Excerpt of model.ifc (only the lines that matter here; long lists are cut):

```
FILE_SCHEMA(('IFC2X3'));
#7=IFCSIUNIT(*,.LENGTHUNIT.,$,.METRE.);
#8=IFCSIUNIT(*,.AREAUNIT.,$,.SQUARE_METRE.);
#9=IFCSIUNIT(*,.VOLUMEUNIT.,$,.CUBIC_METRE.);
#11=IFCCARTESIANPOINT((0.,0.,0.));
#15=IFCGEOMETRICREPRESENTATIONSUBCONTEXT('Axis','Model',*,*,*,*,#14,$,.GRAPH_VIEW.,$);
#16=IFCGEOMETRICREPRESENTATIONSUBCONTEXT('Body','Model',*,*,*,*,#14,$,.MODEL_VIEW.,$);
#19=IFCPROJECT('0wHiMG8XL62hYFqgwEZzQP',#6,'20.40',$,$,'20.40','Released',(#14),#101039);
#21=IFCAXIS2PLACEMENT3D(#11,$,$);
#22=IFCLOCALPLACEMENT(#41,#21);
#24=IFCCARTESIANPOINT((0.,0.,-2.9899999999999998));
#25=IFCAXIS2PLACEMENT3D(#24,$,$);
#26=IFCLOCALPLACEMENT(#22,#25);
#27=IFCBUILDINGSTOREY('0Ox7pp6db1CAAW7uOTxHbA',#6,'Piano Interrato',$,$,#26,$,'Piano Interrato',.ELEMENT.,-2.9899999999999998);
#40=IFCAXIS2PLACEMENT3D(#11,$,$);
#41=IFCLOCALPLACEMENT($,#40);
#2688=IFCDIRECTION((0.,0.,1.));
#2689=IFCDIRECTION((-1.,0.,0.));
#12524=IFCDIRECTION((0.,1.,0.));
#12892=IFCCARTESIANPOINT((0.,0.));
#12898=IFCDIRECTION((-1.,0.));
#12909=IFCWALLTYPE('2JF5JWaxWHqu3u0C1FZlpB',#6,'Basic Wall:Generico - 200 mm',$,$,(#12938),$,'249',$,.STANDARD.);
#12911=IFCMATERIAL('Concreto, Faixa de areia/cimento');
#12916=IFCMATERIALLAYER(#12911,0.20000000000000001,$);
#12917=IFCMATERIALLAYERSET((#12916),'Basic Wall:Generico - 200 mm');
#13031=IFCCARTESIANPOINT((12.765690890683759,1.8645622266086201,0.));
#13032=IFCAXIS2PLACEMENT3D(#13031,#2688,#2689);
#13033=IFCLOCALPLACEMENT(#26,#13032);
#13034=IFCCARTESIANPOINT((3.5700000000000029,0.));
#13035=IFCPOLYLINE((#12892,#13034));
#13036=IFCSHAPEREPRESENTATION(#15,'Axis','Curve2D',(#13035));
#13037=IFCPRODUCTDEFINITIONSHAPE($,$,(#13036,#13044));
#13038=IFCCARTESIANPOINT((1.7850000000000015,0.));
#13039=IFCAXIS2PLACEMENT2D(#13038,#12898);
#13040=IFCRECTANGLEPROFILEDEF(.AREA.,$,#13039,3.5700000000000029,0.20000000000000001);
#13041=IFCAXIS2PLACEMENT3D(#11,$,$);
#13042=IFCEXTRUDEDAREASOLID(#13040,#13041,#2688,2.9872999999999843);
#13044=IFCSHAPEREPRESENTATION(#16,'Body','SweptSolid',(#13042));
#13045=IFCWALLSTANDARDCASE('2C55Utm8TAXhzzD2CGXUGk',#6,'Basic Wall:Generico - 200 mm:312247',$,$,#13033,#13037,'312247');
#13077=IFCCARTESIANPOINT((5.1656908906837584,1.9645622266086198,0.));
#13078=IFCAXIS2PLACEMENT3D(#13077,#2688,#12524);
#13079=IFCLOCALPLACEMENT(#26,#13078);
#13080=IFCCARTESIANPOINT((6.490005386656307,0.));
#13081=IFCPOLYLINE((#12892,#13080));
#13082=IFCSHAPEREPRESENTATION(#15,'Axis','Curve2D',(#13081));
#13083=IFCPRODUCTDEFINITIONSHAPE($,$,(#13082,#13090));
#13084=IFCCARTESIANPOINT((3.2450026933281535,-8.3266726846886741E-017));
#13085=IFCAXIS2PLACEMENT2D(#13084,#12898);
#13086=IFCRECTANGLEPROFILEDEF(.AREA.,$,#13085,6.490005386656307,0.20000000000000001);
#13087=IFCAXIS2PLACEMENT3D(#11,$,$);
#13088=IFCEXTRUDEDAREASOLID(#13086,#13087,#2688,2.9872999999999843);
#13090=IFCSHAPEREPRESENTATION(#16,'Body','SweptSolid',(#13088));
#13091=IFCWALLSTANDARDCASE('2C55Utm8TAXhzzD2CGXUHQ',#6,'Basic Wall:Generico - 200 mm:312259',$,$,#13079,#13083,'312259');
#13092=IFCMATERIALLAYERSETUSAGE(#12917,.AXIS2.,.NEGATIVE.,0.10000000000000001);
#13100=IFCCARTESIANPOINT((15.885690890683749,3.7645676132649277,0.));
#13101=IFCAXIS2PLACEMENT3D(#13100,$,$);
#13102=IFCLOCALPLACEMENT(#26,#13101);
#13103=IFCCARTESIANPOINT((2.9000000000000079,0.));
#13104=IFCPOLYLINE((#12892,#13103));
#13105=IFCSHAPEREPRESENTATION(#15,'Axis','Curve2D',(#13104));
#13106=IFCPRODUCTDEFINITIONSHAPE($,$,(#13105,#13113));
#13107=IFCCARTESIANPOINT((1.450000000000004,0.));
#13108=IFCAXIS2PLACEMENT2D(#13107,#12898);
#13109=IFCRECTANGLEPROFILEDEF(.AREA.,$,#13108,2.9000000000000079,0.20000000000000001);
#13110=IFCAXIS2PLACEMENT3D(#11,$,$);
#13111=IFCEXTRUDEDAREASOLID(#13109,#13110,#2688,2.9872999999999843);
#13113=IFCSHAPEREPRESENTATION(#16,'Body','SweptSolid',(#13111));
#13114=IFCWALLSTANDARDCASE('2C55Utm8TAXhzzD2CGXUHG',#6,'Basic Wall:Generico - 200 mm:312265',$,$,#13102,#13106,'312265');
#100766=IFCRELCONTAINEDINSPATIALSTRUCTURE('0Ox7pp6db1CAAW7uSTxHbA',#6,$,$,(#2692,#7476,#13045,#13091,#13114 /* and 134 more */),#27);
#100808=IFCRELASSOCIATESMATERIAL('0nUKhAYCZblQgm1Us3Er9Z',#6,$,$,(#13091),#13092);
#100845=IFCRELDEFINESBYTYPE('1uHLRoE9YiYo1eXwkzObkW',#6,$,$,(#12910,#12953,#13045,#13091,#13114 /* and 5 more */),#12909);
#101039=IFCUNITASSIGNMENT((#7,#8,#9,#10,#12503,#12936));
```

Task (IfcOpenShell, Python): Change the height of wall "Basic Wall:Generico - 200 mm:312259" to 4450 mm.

```python
import ifcopenshell
import ifcopenshell.geom
import ifcopenshell.util.representation
import ifcopenshell.util.shape
import ifcopenshell.util.unit

model = ifcopenshell.open("model.ifc")
unit_scale = ifcopenshell.util.unit.calculate_unit_scale(model)
settings = ifcopenshell.geom.settings()


def volume(element):
    """Net volume in cubic metres, openings subtracted."""
    shape = ifcopenshell.geom.create_shape(settings, element)
    return ifcopenshell.util.shape.get_volume(shape.geometry)


wall = model.by_guid("2C55Utm8TAXhzzD2CGXUHQ")
before = volume(wall)

body = ifcopenshell.util.representation.get_representation(wall, "Model", "Body")
solid = body.Items[0]
old_height = solid.Depth
solid.Depth = 4.45 / unit_scale
after = volume(wall)

print(f"height {old_height:g} -> {solid.Depth:g}, volume {before:.3f} -> {after:.3f} m3")

model.write("model-out.ifc")
```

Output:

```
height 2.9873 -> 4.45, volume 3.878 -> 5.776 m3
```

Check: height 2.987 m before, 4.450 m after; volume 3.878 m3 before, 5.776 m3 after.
